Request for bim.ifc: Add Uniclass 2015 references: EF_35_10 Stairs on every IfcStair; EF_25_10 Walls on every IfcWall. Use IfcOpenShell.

First a look at what the model holds.

```python
import ifcopenshell

model = ifcopenshell.open("bim.ifc")
print(model.schema)
print("classifications:", [c.Name for c in model.by_type("IfcClassification")])
for ifc_class in ("IfcDoor", "IfcRoof", "IfcStair", "IfcWall", "IfcWindow"):
    print(ifc_class, len(model.by_type(ifc_class)))
```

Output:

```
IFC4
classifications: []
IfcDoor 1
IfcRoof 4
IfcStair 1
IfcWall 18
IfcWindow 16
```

```python
import ifcopenshell
import ifcopenshell.api.classification

model = ifcopenshell.open("bim.ifc")

system = ifcopenshell.api.classification.add_classification(model, classification="Uniclass 2015")

codes = {
    "IfcStair": ("EF_35_10", "Stairs"),
    "IfcWall": ("EF_25_10", "Walls"),
}
for ifc_class, (code, name) in codes.items():
    products = model.by_type(ifc_class)
    ifcopenshell.api.classification.add_reference(
        model, products=products, classification=system, identification=code, name=name
    )
    print(code, len(products))

model.write("bim_v2.ifc")
```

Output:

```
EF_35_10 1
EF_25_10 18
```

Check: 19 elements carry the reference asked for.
